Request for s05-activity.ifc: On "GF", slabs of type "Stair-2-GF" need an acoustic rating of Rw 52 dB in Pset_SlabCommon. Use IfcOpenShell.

First a look at what the model holds.

```python
import ifcopenshell
import ifcopenshell.util.element

model = ifcopenshell.open("s05-activity.ifc")
print(model.schema)
storey = next(s for s in model.by_type("IfcBuildingStorey") if s.Name == "GF")
slabs = [e for e in ifcopenshell.util.element.get_decomposition(storey) if e.is_a("IfcSlab")]
seen = {}
for e in slabs:
    element_type = ifcopenshell.util.element.get_type(e)
    key = (element_type.Name if element_type != e and element_type else None, ifcopenshell.util.element.get_pset(e, "Pset_SlabCommon", "AcousticRating"))
    seen[key] = seen.get(key, 0) + 1
for (name, value), count in sorted(seen.items(), key=str):
    print(count, "x", name, "|", value)
```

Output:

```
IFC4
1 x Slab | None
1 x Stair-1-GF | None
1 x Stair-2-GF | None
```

```python
import ifcopenshell
import ifcopenshell.api.pset
import ifcopenshell.util.element

model = ifcopenshell.open("s05-activity.ifc")

storey = next(s for s in model.by_type("IfcBuildingStorey") if s.Name == "GF")
slabs = [e for e in ifcopenshell.util.element.get_decomposition(storey) if e.is_a("IfcSlab")]

count = 0
for e in slabs:
    element_type = ifcopenshell.util.element.get_type(e)
    if element_type in (None, e) or element_type.Name != "Stair-2-GF":
        continue
    # add_pset returns the element's existing set when there is one.
    pset = ifcopenshell.api.pset.add_pset(model, product=e, name="Pset_SlabCommon")
    ifcopenshell.api.pset.edit_pset(model, pset=pset, properties={"AcousticRating": "Rw 52 dB"})
    count += 1

print(count, "slabs updated")

model.write("s05-activity_rev.ifc")
```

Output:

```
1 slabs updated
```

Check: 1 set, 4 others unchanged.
